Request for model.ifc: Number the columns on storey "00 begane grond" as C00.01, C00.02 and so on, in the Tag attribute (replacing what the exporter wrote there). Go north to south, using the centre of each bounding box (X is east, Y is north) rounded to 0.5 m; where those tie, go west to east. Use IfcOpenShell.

First a look at what the model holds.

```python
import ifcopenshell
import ifcopenshell.util.element
import ifcopenshell.util.placement

model = ifcopenshell.open("model.ifc")
print(model.schema)
storey = next(s for s in model.by_type("IfcBuildingStorey") if s.Name == "00 begane grond")
columns = [e for e in ifcopenshell.util.element.get_decomposition(storey) if e.is_a("IfcColumn")]
for e in sorted(columns, key=lambda e: e.id()):
    origin = ifcopenshell.util.placement.get_local_placement(e.ObjectPlacement)[:3, 3]
    print(e.id(), e.Tag, e.Name, origin.round(2) + 0.0, sep=" | ")
```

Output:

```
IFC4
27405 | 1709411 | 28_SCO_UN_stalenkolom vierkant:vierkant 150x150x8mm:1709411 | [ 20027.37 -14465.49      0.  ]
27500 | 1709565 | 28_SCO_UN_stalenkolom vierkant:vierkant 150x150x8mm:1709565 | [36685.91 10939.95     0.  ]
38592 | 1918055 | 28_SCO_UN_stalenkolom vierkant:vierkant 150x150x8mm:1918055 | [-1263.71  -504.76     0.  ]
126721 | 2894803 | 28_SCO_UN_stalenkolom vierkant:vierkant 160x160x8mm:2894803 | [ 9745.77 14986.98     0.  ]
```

```python
import ifcopenshell
import ifcopenshell.geom
import ifcopenshell.util.element
import ifcopenshell.util.shape

model = ifcopenshell.open("model.ifc")
settings = ifcopenshell.geom.settings()
settings.set("use-world-coords", True)


def centre(element):
    shape = ifcopenshell.geom.create_shape(settings, element)
    return ifcopenshell.util.shape.get_bbox_centroid(shape.geometry)


storey = next(s for s in model.by_type("IfcBuildingStorey") if s.Name == "00 begane grond")
columns = [e for e in ifcopenshell.util.element.get_decomposition(storey) if e.is_a("IfcColumn")]

# Insertion points can sit at a corner or the storey origin, so sort by the geometry (in metres).
centres = {e: centre(e) for e in columns}
columns.sort(key=lambda e: (-round(centres[e][1] / 0.5), centres[e][0]))

for i, e in enumerate(columns, start=1):
    number = f"C00.{i:02d}"
    e.Tag = number
    print(e.id(), number)

model.write("model_updated.ifc")
```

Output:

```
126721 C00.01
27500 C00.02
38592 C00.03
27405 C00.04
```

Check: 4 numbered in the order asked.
